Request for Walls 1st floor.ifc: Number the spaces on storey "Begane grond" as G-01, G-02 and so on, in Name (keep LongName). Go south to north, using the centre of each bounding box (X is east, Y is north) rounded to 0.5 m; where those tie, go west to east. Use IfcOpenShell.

First a look at what the model holds.

```python
import ifcopenshell
import ifcopenshell.util.element
import ifcopenshell.util.placement

model = ifcopenshell.open("Walls 1st floor.ifc")
print(model.schema)
storey = next(s for s in model.by_type("IfcBuildingStorey") if s.Name == "Begane grond")
spaces = [e for e in ifcopenshell.util.element.get_decomposition(storey) if e.is_a("IfcSpace")]
for e in sorted(spaces, key=lambda e: e.id()):
    origin = ifcopenshell.util.placement.get_local_placement(e.ObjectPlacement)[:3, 3]
    print(e.id(), e.Name, e.LongName, origin.round(2) + 0.0, sep=" | ")
```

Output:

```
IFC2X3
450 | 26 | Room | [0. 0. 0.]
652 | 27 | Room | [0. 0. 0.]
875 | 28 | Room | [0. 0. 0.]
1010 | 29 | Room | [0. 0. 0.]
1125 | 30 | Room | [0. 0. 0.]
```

```python
import ifcopenshell
import ifcopenshell.geom
import ifcopenshell.util.element
import ifcopenshell.util.shape

model = ifcopenshell.open("Walls 1st floor.ifc")
settings = ifcopenshell.geom.settings()
settings.set("use-world-coords", True)


def centre(element):
    shape = ifcopenshell.geom.create_shape(settings, element)
    return ifcopenshell.util.shape.get_bbox_centroid(shape.geometry)


storey = next(s for s in model.by_type("IfcBuildingStorey") if s.Name == "Begane grond")
spaces = [e for e in ifcopenshell.util.element.get_decomposition(storey) if e.is_a("IfcSpace")]

# Insertion points can sit at a corner or the storey origin, so sort by the geometry (in metres).
centres = {e: centre(e) for e in spaces}
spaces.sort(key=lambda e: (round(centres[e][1] / 0.5), centres[e][0]))

for i, e in enumerate(spaces, start=1):
    number = f"G-{i:02d}"
    e.Name = number
    print(e.id(), number)

model.write("Walls 1st floor_v2.ifc")
```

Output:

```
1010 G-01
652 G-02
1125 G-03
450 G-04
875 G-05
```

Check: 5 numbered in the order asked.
